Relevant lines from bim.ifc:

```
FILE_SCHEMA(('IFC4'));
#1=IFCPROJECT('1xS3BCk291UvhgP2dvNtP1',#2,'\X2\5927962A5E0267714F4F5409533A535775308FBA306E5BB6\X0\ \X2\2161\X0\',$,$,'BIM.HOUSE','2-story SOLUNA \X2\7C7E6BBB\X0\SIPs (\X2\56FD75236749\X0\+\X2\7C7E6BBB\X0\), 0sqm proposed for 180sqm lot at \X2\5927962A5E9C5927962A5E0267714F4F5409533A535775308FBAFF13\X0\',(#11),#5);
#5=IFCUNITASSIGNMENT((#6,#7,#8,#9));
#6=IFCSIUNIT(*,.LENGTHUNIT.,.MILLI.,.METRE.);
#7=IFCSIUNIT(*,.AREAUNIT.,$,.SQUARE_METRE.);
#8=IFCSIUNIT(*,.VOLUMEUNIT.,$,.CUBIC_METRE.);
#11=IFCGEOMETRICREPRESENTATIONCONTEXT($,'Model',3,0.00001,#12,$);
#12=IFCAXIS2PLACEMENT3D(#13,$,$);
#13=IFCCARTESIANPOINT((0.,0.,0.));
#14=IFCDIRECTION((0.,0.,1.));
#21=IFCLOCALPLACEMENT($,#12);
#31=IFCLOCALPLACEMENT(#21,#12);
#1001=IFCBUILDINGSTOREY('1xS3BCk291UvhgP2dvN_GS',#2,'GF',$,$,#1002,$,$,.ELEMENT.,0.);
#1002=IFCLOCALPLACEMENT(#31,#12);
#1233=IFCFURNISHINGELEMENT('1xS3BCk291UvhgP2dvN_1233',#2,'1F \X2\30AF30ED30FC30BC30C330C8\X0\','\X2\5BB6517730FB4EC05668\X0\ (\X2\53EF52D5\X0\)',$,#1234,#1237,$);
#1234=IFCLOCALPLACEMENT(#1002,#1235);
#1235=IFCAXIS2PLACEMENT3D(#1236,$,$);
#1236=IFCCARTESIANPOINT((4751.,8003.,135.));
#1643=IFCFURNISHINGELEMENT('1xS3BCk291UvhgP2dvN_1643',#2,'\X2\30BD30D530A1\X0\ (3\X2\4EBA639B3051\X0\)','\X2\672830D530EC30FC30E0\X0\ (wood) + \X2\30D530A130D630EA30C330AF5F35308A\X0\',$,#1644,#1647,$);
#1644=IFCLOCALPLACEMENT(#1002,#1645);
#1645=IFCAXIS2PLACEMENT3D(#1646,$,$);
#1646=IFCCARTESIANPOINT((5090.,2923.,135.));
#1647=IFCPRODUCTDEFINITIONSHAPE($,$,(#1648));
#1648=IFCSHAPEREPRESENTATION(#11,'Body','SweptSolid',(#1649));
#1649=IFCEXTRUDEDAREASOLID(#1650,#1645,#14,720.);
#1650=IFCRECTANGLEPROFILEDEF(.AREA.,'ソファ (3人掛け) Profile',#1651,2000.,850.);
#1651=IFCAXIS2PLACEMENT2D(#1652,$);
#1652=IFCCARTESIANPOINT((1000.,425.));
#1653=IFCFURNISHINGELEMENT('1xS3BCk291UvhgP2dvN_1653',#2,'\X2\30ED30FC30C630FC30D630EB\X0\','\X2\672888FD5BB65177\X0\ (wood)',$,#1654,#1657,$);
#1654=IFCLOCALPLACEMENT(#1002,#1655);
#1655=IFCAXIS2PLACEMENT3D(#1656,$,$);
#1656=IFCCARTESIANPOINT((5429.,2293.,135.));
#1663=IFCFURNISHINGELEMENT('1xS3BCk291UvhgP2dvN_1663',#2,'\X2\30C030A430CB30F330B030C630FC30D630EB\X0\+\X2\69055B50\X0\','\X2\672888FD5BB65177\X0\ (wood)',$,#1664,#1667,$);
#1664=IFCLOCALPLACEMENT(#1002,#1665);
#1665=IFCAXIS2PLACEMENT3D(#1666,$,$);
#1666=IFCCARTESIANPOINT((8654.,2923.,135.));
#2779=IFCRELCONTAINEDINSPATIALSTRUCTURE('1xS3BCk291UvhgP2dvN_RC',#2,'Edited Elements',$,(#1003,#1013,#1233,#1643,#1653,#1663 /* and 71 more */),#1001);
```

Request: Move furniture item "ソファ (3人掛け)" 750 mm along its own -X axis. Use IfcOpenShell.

```python
import ifcopenshell
import ifcopenshell.api.geometry
import ifcopenshell.util.placement

model = ifcopenshell.open("bim.ifc")

item = model.by_guid("1xS3BCk291UvhgP2dvN_1643")
matrix = ifcopenshell.util.placement.get_local_placement(item.ObjectPlacement)
matrix[:3, 3] -= matrix[:3, 0] * 750.0
ifcopenshell.api.geometry.edit_object_placement(model, product=item, matrix=matrix, is_si=False)

print(ifcopenshell.util.placement.get_local_placement(item.ObjectPlacement).round(3) + 0.0)

model.write("bim_rev.ifc")
```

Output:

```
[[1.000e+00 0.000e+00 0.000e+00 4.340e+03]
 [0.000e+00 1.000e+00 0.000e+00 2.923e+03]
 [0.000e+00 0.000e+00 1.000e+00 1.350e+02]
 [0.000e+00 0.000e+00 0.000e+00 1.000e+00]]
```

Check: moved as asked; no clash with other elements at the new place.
